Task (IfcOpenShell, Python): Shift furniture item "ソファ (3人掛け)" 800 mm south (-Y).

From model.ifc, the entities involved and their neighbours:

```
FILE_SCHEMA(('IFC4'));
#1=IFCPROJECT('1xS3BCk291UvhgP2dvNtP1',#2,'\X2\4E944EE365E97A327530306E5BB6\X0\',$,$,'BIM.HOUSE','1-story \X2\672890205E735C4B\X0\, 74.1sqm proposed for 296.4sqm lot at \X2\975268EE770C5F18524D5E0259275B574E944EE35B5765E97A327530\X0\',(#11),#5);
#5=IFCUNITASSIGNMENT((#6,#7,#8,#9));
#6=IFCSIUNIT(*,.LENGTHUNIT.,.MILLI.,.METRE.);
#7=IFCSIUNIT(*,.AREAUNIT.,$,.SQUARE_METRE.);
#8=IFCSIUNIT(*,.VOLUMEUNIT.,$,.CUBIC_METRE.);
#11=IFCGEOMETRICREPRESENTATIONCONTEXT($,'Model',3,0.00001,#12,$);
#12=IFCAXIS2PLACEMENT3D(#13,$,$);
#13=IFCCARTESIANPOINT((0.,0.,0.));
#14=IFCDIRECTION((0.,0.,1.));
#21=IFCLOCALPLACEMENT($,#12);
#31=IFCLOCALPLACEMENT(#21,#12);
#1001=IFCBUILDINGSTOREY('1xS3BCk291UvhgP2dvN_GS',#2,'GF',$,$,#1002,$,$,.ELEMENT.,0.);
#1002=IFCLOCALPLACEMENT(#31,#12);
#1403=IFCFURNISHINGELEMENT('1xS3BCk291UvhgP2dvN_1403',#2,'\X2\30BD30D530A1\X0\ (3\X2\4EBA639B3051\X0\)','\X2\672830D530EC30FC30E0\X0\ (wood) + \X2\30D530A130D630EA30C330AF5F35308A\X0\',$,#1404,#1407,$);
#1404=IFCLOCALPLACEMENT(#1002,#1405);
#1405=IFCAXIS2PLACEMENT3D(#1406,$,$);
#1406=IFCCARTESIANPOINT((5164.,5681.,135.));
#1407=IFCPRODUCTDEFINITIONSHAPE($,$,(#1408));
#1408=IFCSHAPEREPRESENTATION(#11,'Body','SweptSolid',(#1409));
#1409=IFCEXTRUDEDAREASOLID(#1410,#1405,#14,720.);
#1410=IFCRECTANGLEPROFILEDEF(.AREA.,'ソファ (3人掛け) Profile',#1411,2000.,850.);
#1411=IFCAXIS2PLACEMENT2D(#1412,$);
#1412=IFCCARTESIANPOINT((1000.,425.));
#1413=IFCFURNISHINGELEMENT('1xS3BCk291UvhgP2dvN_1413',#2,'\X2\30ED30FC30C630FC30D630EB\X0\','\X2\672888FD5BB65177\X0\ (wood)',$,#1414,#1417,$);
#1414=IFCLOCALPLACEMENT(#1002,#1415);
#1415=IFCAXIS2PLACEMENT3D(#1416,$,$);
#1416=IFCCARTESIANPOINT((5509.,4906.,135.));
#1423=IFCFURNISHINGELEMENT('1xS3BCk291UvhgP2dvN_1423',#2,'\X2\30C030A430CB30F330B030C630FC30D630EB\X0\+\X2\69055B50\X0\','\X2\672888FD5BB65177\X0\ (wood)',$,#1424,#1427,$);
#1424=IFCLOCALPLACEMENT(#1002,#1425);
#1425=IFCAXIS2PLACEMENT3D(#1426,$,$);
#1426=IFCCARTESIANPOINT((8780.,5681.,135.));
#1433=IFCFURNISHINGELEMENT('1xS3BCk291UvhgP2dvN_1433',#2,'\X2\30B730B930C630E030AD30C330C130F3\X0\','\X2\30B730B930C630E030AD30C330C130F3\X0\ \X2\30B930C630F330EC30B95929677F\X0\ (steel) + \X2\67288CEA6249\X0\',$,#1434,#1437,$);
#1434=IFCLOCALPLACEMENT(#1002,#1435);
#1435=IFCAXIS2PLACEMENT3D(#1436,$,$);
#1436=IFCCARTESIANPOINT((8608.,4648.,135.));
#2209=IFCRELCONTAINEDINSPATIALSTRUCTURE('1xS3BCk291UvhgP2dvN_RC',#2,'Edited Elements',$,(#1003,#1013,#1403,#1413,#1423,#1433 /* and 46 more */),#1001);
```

```python
import ifcopenshell
import ifcopenshell.api.geometry
import ifcopenshell.util.placement
import ifcopenshell.util.unit

model = ifcopenshell.open("model.ifc")
unit_scale = ifcopenshell.util.unit.calculate_unit_scale(model)

item = model.by_guid("1xS3BCk291UvhgP2dvN_1403")
matrix = ifcopenshell.util.placement.get_local_placement(item.ObjectPlacement)
matrix[1, 3] -= 0.8 / unit_scale
ifcopenshell.api.geometry.edit_object_placement(model, product=item, matrix=matrix, is_si=False)

print(ifcopenshell.util.placement.get_local_placement(item.ObjectPlacement).round(3) + 0.0)

model.write("model-out.ifc")
```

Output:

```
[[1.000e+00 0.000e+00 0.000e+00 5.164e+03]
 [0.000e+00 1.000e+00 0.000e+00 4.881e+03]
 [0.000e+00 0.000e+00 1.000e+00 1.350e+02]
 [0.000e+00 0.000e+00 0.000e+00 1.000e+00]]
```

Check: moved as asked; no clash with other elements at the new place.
